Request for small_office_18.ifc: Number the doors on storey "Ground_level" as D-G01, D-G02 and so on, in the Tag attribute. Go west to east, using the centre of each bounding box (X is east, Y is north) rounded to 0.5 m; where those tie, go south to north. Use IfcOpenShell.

First a look at what the model holds.

```python
import ifcopenshell
import ifcopenshell.util.element
import ifcopenshell.util.placement

model = ifcopenshell.open("small_office_18.ifc")
print(model.schema)
storey = next(s for s in model.by_type("IfcBuildingStorey") if s.Name == "Ground_level")
doors = [e for e in ifcopenshell.util.element.get_decomposition(storey) if e.is_a("IfcDoor")]
for e in sorted(doors, key=lambda e: e.id()):
    origin = ifcopenshell.util.placement.get_local_placement(e.ObjectPlacement)[:3, 3]
    print(e.id(), e.Tag, e.Name, origin.round(2) + 0.0, sep=" | ")
```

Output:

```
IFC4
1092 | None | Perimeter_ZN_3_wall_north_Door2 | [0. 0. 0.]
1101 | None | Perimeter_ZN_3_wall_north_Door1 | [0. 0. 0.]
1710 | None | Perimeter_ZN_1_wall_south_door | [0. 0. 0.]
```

```python
import ifcopenshell
import ifcopenshell.geom
import ifcopenshell.util.element
import ifcopenshell.util.shape

model = ifcopenshell.open("small_office_18.ifc")
settings = ifcopenshell.geom.settings()
settings.set("use-world-coords", True)


def centre(element):
    shape = ifcopenshell.geom.create_shape(settings, element)
    return ifcopenshell.util.shape.get_bbox_centroid(shape.geometry)


storey = next(s for s in model.by_type("IfcBuildingStorey") if s.Name == "Ground_level")
doors = [e for e in ifcopenshell.util.element.get_decomposition(storey) if e.is_a("IfcDoor")]

# Insertion points can sit at a corner or the storey origin, so sort by the geometry (in metres).
centres = {e: centre(e) for e in doors}
doors.sort(key=lambda e: (round(centres[e][0] / 0.5), centres[e][1]))

for i, e in enumerate(doors, start=1):
    number = f"D-G{i:02d}"
    e.Tag = number
    print(e.id(), number)

model.write("small_office_18_v2.ifc")
```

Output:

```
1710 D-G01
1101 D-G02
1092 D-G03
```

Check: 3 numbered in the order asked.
